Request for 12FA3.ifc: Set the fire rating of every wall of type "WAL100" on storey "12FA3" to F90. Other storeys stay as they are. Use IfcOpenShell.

First a look at what the model holds.

```python
import ifcopenshell
import ifcopenshell.util.element

model = ifcopenshell.open("12FA3.ifc")
print(model.schema)
storey = next(s for s in model.by_type("IfcBuildingStorey") if s.Name == "12FA3")
walls = [e for e in ifcopenshell.util.element.get_decomposition(storey) if e.is_a("IfcWall")]
seen = {}
for e in walls:
    element_type = ifcopenshell.util.element.get_type(e)
    key = (element_type.Name if element_type != e and element_type else None, ifcopenshell.util.element.get_pset(e, "Pset_WallCommon", "FireRating"))
    seen[key] = seen.get(key, 0) + 1
for (name, value), count in sorted(seen.items(), key=str):
    print(count, "x", name, "|", value)
```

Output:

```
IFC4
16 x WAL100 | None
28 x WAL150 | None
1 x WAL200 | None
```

```python
import ifcopenshell
import ifcopenshell.api.pset
import ifcopenshell.util.element

model = ifcopenshell.open("12FA3.ifc")

storey = next(s for s in model.by_type("IfcBuildingStorey") if s.Name == "12FA3")
walls = [e for e in ifcopenshell.util.element.get_decomposition(storey) if e.is_a("IfcWall")]

count = 0
for e in walls:
    element_type = ifcopenshell.util.element.get_type(e)
    if element_type in (None, e) or element_type.Name != "WAL100":
        continue
    # add_pset returns the element's existing set when there is one.
    pset = ifcopenshell.api.pset.add_pset(model, product=e, name="Pset_WallCommon")
    ifcopenshell.api.pset.edit_pset(model, pset=pset, properties={"FireRating": "F90"})
    count += 1

print(count, "walls updated")

model.write("12FA3_updated.ifc")
```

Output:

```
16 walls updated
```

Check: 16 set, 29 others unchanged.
